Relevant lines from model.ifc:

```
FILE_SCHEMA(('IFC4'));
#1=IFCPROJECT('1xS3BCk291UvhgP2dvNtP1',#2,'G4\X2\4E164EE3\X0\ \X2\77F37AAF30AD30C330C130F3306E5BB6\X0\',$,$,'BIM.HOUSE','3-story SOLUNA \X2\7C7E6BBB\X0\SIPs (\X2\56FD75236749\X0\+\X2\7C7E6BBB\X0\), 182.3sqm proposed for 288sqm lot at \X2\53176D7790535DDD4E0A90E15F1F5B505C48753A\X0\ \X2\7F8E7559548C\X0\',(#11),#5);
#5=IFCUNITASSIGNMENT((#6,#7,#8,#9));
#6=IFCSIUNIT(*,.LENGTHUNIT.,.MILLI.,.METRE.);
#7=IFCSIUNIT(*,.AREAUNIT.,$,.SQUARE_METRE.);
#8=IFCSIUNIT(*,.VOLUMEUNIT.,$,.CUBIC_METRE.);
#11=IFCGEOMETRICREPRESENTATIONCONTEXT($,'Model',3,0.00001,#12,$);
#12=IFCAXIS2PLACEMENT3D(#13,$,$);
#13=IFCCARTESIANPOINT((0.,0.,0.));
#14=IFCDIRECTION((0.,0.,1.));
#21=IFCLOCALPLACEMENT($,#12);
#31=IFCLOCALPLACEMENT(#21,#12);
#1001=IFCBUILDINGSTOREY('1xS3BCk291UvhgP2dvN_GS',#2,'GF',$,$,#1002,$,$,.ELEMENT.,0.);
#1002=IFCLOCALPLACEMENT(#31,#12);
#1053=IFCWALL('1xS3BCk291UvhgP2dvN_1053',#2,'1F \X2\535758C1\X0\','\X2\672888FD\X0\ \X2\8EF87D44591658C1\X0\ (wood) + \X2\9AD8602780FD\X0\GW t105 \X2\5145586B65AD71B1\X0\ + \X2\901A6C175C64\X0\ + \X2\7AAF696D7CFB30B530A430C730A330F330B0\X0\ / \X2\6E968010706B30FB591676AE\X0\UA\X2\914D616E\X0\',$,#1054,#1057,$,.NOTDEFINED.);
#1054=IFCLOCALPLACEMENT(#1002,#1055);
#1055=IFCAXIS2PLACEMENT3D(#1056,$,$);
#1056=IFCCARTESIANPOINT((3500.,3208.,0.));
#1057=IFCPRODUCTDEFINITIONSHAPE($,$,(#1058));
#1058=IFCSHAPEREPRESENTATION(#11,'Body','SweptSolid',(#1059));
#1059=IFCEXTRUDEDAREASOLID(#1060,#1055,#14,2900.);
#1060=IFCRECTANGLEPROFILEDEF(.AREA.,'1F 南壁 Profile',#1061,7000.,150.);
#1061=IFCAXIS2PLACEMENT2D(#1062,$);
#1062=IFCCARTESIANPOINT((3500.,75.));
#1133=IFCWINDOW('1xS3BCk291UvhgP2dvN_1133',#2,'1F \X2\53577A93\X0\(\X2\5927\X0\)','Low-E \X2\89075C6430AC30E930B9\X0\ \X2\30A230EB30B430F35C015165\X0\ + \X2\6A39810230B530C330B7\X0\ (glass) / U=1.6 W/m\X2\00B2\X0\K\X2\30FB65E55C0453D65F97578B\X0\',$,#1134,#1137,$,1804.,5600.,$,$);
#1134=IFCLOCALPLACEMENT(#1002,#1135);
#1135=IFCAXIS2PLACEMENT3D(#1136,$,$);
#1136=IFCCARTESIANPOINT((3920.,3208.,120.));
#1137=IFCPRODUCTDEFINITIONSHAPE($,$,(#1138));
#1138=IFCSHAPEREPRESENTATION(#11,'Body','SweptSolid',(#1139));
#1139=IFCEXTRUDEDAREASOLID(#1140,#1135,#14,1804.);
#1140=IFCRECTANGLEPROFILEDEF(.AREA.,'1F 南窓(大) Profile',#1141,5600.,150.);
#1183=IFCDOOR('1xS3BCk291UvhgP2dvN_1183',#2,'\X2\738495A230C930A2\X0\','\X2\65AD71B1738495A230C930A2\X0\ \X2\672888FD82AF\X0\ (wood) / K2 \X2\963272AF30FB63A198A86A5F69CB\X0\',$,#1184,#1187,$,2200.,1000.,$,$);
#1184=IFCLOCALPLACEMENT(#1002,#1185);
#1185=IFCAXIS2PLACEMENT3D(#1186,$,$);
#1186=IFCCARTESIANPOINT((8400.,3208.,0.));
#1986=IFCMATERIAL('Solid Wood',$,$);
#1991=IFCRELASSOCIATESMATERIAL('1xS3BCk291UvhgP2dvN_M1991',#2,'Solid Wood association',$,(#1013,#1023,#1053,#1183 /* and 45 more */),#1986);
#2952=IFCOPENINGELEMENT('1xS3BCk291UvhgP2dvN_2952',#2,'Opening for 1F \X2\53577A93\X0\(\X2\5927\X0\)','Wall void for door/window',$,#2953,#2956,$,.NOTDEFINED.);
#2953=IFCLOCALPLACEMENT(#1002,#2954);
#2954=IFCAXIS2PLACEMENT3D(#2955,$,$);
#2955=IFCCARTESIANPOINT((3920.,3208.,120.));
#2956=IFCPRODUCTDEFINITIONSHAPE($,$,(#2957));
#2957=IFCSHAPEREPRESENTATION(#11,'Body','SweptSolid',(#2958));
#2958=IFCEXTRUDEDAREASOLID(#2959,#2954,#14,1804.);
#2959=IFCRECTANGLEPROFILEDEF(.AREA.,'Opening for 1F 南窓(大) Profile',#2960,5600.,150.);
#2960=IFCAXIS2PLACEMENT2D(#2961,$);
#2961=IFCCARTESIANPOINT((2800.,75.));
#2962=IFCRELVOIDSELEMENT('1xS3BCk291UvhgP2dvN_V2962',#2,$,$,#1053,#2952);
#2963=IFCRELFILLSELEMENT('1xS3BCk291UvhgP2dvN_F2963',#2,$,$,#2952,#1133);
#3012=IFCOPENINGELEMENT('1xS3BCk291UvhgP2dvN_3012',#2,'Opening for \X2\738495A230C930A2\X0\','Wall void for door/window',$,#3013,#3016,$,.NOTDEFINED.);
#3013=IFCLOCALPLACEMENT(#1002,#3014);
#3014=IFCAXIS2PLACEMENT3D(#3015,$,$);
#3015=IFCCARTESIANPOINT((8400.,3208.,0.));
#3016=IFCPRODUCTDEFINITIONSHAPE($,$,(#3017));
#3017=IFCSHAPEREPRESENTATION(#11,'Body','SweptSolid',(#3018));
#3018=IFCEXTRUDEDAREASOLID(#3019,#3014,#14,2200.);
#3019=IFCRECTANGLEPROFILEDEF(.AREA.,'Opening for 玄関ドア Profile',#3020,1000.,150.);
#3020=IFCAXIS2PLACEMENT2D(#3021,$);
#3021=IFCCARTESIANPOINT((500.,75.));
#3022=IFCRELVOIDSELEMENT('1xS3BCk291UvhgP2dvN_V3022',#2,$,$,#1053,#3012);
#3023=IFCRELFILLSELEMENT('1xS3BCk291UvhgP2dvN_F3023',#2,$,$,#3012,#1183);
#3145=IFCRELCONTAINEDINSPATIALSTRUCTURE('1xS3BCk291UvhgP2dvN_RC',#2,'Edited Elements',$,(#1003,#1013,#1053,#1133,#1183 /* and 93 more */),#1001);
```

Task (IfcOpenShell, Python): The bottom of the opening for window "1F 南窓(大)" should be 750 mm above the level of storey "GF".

```python
import numpy as np
import ifcopenshell
import ifcopenshell.api.geometry
import ifcopenshell.geom
import ifcopenshell.util.element
import ifcopenshell.util.placement
import ifcopenshell.util.shape
import ifcopenshell.util.unit

model = ifcopenshell.open("model.ifc")
unit_scale = ifcopenshell.util.unit.calculate_unit_scale(model)

window = model.by_guid("1xS3BCk291UvhgP2dvN_1133")
opening = window.FillsVoids[0].RelatingOpeningElement
storey = ifcopenshell.util.element.get_container(window, ifc_class="IfcBuildingStorey")
level = ifcopenshell.util.placement.get_local_placement(storey.ObjectPlacement)[2, 3]

# The opening's origin need not be at the sill, so measure its lowest point.
shape = ifcopenshell.geom.create_shape(ifcopenshell.geom.settings(), opening)
bottom = ifcopenshell.util.shape.get_shape_bottom_elevation(shape, shape.geometry) / unit_scale
dz = level + 0.75 / unit_scale - bottom

shift = np.array([0.0, 0.0, dz])
# The window is not placed relative to its opening, so move both.
for product in (opening, window):
    matrix = ifcopenshell.util.placement.get_local_placement(product.ObjectPlacement)
    matrix[:3, 3] += shift
    ifcopenshell.api.geometry.edit_object_placement(model, product=product, matrix=matrix, is_si=False)

print(f"moved by {dz * unit_scale:+.3f} m")

model.write("model_updated.ifc")
```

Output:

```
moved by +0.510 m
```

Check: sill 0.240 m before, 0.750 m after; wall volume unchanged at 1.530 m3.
